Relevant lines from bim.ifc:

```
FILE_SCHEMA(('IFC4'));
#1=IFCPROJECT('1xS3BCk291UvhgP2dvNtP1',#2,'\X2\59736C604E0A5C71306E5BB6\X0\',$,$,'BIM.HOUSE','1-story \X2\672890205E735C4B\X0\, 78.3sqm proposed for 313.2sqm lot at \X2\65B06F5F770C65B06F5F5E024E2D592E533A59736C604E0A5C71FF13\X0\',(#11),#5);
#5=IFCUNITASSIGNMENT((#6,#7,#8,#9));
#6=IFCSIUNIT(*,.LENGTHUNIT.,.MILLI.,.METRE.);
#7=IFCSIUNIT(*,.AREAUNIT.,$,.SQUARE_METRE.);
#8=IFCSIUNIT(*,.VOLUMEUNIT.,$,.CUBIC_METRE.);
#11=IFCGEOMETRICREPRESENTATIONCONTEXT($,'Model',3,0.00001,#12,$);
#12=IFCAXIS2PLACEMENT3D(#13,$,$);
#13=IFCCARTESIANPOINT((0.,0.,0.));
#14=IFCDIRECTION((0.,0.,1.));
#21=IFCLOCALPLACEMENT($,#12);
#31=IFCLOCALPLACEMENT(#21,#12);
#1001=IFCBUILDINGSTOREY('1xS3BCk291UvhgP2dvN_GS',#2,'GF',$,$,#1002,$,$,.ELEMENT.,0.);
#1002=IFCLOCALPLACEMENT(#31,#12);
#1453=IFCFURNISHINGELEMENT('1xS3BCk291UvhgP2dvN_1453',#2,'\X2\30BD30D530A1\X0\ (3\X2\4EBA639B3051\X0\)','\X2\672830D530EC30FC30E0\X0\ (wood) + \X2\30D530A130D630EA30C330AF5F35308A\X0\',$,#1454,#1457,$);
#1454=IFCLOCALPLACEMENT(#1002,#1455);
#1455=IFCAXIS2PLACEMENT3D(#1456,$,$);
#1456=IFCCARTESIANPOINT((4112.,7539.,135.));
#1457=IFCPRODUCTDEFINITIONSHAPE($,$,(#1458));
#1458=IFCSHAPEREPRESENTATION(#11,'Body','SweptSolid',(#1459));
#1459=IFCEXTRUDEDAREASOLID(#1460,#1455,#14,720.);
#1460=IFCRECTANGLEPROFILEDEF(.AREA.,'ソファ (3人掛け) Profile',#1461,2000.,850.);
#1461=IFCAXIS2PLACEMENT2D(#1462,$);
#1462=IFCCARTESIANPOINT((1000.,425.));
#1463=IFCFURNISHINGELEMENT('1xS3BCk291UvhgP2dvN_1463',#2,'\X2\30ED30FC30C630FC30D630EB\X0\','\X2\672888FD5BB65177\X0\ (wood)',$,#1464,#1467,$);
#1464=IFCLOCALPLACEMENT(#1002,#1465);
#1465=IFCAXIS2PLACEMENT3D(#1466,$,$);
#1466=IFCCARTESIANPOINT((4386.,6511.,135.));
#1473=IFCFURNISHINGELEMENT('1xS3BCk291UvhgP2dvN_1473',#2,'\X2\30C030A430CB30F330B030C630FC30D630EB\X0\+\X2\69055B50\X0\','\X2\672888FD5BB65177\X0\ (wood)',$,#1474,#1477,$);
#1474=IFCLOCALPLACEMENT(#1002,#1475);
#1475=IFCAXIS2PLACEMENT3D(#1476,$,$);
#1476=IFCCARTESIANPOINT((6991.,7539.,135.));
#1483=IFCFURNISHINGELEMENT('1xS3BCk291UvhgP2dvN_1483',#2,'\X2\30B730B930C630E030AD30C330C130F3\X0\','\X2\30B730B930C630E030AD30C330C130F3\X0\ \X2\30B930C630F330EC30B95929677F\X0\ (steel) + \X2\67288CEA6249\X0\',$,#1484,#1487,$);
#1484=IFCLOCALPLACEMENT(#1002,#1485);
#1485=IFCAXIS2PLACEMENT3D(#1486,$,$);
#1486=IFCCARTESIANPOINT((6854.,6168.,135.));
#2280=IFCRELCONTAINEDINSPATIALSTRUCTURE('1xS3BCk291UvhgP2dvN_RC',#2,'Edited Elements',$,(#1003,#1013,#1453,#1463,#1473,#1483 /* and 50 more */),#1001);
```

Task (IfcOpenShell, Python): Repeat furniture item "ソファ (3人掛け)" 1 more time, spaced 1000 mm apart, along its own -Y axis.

```python
import ifcopenshell
import ifcopenshell.api.geometry
import ifcopenshell.api.root
import ifcopenshell.util.element
import ifcopenshell.util.placement
import ifcopenshell.util.unit

model = ifcopenshell.open("bim.ifc")
unit_scale = ifcopenshell.util.unit.calculate_unit_scale(model)


def reuse_history(source, copy):
    """copy_class also copies each property set's owner history, people and application; keep the originals."""
    for rel in copy.IsDefinedBy:
        if rel.is_a("IfcRelDefinesByProperties") and (history := rel.RelatingPropertyDefinition.OwnerHistory):
            rel.RelatingPropertyDefinition.OwnerHistory = source.OwnerHistory
            ifcopenshell.util.element.remove_deep2(model, history)


source = model.by_id(1453)
base = ifcopenshell.util.placement.get_local_placement(source.ObjectPlacement)
step = -base[:3, 1] * 1 / unit_scale

for i in range(1, 2):
    copy = ifcopenshell.api.root.copy_class(model, product=source)
    copy.Representation = ifcopenshell.util.element.copy_deep(
        model, source.Representation, exclude=["IfcGeometricRepresentationContext", "IfcRepresentationMap"]
    )
    reuse_history(source, copy)
    matrix = base.copy()
    matrix[:3, 3] += i * step
    print("added at", matrix[:3, 3].round(3) + 0.0)
    ifcopenshell.api.geometry.edit_object_placement(model, product=copy, matrix=matrix, is_si=False)

model.write("bim_updated.ifc")
```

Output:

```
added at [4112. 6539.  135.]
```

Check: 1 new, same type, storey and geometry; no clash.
